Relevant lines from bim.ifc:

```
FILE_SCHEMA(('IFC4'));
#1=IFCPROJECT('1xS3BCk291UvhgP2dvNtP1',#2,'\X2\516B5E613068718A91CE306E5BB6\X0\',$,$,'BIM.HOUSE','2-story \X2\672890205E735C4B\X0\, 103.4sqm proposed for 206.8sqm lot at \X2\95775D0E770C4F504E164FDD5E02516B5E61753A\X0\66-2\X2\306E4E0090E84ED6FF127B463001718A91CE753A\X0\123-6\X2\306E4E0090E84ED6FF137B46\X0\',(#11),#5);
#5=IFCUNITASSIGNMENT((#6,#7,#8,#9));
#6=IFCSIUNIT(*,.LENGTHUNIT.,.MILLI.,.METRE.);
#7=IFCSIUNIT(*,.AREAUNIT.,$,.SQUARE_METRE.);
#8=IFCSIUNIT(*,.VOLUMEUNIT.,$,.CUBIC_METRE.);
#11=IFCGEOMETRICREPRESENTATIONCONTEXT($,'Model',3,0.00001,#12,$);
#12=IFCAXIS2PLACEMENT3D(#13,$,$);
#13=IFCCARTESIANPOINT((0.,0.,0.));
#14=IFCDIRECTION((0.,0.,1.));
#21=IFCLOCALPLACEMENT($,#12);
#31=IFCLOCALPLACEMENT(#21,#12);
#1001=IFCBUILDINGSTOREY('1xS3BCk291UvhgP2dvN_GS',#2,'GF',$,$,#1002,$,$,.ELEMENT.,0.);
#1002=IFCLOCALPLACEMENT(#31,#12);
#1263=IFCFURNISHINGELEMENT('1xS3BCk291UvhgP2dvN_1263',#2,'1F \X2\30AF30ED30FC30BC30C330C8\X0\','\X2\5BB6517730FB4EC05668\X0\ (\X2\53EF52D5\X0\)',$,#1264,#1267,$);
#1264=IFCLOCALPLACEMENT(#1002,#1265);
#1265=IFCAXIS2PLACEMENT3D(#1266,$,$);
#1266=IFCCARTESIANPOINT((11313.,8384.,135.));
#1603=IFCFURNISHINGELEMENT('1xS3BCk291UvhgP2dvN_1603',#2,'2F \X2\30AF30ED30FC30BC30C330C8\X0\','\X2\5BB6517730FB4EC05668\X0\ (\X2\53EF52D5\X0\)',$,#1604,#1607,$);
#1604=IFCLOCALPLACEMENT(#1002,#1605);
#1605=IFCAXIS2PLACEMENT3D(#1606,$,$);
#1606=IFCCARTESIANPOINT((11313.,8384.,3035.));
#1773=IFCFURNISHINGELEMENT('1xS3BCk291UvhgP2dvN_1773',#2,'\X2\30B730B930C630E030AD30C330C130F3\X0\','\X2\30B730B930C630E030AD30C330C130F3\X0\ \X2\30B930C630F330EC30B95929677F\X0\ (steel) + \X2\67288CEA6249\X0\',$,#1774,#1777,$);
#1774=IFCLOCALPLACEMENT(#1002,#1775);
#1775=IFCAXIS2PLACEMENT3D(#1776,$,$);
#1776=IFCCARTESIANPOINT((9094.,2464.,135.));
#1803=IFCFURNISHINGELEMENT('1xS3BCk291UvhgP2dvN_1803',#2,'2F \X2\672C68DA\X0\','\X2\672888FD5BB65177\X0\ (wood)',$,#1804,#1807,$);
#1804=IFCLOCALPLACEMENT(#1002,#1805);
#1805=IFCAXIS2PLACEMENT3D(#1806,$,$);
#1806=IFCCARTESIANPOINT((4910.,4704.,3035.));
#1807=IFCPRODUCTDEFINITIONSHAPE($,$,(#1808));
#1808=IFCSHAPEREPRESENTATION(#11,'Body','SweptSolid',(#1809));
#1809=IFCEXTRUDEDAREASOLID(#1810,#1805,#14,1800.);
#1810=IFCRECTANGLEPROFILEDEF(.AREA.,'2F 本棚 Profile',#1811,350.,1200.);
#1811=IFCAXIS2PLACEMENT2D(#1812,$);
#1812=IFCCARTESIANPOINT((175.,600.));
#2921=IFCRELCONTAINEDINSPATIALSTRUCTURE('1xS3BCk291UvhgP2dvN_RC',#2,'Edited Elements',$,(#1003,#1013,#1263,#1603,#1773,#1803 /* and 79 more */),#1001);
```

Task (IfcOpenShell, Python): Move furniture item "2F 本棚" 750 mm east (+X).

```python
import ifcopenshell
import ifcopenshell.api.geometry
import ifcopenshell.util.placement
import ifcopenshell.util.unit

model = ifcopenshell.open("bim.ifc")
unit_scale = ifcopenshell.util.unit.calculate_unit_scale(model)

item = model.by_guid("1xS3BCk291UvhgP2dvN_1803")
matrix = ifcopenshell.util.placement.get_local_placement(item.ObjectPlacement)
matrix[0, 3] += 0.75 / unit_scale
ifcopenshell.api.geometry.edit_object_placement(model, product=item, matrix=matrix, is_si=False)

print(ifcopenshell.util.placement.get_local_placement(item.ObjectPlacement).round(3) + 0.0)

model.write("bim_rev.ifc")
```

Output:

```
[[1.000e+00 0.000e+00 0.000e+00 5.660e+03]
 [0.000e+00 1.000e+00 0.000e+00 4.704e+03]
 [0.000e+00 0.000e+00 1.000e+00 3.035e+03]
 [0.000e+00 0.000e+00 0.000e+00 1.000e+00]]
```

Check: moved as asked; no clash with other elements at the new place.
